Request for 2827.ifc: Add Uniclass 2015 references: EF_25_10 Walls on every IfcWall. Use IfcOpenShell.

First a look at what the model holds.

```python
import ifcopenshell

model = ifcopenshell.open("2827.ifc")
print(model.schema)
print("classifications:", [c.Name for c in model.by_type("IfcClassification")])
for ifc_class in ("IfcDoor", "IfcRoof", "IfcStair", "IfcWall", "IfcWindow"):
    print(ifc_class, len(model.by_type(ifc_class)))
```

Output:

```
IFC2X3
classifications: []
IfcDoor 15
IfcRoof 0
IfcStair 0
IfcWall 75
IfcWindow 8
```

```python
import ifcopenshell
import ifcopenshell.api.classification

model = ifcopenshell.open("2827.ifc")

# IFC2X3 requires Source and Edition and has no link from the project to the system.
system = model.create_entity("IfcClassification", Source="NBS", Edition="2015", Name="Uniclass 2015")

codes = {
    "IfcWall": ("EF_25_10", "Walls"),
}
for ifc_class, (code, name) in codes.items():
    products = model.by_type(ifc_class)
    ifcopenshell.api.classification.add_reference(
        model, products=products, classification=system, identification=code, name=name
    )
    print(code, len(products))

model.write("2827_rev.ifc")
```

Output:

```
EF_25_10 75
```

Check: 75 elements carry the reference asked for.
